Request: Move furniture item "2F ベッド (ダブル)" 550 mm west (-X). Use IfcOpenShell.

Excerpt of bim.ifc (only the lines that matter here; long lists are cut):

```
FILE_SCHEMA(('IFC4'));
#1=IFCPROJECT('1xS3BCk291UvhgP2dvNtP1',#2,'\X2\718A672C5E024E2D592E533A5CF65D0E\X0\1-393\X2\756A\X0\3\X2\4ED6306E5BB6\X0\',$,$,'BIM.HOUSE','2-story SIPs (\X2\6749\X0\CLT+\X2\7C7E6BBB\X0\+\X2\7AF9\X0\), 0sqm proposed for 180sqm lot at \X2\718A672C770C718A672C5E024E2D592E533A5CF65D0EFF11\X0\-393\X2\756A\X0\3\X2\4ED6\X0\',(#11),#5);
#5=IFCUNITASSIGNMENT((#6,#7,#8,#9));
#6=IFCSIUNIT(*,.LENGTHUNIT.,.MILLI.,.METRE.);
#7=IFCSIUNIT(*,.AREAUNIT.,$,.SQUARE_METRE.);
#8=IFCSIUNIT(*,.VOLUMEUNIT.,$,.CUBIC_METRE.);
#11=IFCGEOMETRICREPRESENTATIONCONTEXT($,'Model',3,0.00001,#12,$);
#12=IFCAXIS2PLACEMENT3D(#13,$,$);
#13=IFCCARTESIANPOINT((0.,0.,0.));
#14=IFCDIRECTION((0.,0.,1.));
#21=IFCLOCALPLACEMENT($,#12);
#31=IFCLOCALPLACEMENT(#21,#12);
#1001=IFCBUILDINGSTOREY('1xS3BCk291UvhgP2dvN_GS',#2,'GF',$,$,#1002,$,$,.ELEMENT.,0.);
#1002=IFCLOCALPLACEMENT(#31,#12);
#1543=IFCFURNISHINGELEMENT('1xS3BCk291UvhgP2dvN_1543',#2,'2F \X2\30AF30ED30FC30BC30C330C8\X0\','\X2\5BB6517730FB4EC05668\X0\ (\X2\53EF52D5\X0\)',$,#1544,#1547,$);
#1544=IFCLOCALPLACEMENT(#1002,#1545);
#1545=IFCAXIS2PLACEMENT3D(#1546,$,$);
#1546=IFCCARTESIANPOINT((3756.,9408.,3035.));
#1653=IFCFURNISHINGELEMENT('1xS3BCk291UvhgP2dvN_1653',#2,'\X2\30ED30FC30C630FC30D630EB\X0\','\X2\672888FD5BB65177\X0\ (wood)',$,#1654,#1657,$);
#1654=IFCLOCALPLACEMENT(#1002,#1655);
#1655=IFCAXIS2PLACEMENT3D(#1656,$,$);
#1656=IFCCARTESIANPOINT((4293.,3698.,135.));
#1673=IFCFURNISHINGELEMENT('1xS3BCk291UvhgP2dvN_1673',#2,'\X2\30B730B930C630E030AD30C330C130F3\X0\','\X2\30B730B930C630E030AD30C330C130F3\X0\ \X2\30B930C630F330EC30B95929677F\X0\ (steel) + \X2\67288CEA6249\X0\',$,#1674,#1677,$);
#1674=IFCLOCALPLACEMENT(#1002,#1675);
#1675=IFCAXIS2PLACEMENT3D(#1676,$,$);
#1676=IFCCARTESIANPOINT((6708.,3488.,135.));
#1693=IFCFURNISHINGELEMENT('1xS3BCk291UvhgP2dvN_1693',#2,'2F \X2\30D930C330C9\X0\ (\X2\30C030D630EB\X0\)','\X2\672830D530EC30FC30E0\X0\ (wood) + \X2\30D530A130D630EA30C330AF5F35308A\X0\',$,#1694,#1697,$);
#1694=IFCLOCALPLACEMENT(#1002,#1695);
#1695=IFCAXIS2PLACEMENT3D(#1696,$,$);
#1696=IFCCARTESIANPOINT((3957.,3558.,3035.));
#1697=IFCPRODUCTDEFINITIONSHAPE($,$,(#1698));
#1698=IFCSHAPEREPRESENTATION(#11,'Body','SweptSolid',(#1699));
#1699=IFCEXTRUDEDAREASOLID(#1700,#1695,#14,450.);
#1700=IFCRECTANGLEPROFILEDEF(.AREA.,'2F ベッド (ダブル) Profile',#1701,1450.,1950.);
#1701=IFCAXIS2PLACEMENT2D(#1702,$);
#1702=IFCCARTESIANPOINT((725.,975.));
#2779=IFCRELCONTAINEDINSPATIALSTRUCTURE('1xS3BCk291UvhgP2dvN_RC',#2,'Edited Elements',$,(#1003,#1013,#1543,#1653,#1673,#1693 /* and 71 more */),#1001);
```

```python
import ifcopenshell
import ifcopenshell.api.geometry
import ifcopenshell.util.placement
import ifcopenshell.util.unit

model = ifcopenshell.open("bim.ifc")
unit_scale = ifcopenshell.util.unit.calculate_unit_scale(model)

item = model.by_id(1693)
matrix = ifcopenshell.util.placement.get_local_placement(item.ObjectPlacement)
matrix[0, 3] -= 0.55 / unit_scale
ifcopenshell.api.geometry.edit_object_placement(model, product=item, matrix=matrix, is_si=False)

print(ifcopenshell.util.placement.get_local_placement(item.ObjectPlacement).round(3) + 0.0)

model.write("bim_v2.ifc")
```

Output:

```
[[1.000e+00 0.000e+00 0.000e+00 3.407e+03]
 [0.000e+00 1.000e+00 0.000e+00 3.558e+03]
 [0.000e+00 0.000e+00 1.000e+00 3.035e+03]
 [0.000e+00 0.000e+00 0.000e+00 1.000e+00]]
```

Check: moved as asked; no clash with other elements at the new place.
